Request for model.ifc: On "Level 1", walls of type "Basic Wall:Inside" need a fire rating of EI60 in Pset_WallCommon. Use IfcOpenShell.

First a look at what the model holds.

```python
import ifcopenshell
import ifcopenshell.util.element

model = ifcopenshell.open("model.ifc")
print(model.schema)
storey = next(s for s in model.by_type("IfcBuildingStorey") if s.Name == "Level 1")
walls = [e for e in ifcopenshell.util.element.get_decomposition(storey) if e.is_a("IfcWall")]
seen = {}
for e in walls:
    element_type = ifcopenshell.util.element.get_type(e)
    key = (element_type.Name if element_type != e and element_type else None, ifcopenshell.util.element.get_pset(e, "Pset_WallCommon", "FireRating"))
    seen[key] = seen.get(key, 0) + 1
for (name, value), count in sorted(seen.items(), key=str):
    print(count, "x", name, "|", value)
```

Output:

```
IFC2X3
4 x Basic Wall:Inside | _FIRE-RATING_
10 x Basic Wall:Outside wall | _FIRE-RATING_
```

```python
import ifcopenshell
import ifcopenshell.api.pset
import ifcopenshell.util.element

model = ifcopenshell.open("model.ifc")

storey = next(s for s in model.by_type("IfcBuildingStorey") if s.Name == "Level 1")
walls = [e for e in ifcopenshell.util.element.get_decomposition(storey) if e.is_a("IfcWall")]

count = 0
for e in walls:
    element_type = ifcopenshell.util.element.get_type(e)
    if element_type in (None, e) or element_type.Name != "Basic Wall:Inside":
        continue
    # add_pset returns the element's existing set when there is one.
    pset = ifcopenshell.api.pset.add_pset(model, product=e, name="Pset_WallCommon")
    ifcopenshell.api.pset.edit_pset(model, pset=pset, properties={"FireRating": "EI60"})
    count += 1

print(count, "walls updated")

model.write("model-out.ifc")
```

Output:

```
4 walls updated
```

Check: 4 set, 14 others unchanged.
